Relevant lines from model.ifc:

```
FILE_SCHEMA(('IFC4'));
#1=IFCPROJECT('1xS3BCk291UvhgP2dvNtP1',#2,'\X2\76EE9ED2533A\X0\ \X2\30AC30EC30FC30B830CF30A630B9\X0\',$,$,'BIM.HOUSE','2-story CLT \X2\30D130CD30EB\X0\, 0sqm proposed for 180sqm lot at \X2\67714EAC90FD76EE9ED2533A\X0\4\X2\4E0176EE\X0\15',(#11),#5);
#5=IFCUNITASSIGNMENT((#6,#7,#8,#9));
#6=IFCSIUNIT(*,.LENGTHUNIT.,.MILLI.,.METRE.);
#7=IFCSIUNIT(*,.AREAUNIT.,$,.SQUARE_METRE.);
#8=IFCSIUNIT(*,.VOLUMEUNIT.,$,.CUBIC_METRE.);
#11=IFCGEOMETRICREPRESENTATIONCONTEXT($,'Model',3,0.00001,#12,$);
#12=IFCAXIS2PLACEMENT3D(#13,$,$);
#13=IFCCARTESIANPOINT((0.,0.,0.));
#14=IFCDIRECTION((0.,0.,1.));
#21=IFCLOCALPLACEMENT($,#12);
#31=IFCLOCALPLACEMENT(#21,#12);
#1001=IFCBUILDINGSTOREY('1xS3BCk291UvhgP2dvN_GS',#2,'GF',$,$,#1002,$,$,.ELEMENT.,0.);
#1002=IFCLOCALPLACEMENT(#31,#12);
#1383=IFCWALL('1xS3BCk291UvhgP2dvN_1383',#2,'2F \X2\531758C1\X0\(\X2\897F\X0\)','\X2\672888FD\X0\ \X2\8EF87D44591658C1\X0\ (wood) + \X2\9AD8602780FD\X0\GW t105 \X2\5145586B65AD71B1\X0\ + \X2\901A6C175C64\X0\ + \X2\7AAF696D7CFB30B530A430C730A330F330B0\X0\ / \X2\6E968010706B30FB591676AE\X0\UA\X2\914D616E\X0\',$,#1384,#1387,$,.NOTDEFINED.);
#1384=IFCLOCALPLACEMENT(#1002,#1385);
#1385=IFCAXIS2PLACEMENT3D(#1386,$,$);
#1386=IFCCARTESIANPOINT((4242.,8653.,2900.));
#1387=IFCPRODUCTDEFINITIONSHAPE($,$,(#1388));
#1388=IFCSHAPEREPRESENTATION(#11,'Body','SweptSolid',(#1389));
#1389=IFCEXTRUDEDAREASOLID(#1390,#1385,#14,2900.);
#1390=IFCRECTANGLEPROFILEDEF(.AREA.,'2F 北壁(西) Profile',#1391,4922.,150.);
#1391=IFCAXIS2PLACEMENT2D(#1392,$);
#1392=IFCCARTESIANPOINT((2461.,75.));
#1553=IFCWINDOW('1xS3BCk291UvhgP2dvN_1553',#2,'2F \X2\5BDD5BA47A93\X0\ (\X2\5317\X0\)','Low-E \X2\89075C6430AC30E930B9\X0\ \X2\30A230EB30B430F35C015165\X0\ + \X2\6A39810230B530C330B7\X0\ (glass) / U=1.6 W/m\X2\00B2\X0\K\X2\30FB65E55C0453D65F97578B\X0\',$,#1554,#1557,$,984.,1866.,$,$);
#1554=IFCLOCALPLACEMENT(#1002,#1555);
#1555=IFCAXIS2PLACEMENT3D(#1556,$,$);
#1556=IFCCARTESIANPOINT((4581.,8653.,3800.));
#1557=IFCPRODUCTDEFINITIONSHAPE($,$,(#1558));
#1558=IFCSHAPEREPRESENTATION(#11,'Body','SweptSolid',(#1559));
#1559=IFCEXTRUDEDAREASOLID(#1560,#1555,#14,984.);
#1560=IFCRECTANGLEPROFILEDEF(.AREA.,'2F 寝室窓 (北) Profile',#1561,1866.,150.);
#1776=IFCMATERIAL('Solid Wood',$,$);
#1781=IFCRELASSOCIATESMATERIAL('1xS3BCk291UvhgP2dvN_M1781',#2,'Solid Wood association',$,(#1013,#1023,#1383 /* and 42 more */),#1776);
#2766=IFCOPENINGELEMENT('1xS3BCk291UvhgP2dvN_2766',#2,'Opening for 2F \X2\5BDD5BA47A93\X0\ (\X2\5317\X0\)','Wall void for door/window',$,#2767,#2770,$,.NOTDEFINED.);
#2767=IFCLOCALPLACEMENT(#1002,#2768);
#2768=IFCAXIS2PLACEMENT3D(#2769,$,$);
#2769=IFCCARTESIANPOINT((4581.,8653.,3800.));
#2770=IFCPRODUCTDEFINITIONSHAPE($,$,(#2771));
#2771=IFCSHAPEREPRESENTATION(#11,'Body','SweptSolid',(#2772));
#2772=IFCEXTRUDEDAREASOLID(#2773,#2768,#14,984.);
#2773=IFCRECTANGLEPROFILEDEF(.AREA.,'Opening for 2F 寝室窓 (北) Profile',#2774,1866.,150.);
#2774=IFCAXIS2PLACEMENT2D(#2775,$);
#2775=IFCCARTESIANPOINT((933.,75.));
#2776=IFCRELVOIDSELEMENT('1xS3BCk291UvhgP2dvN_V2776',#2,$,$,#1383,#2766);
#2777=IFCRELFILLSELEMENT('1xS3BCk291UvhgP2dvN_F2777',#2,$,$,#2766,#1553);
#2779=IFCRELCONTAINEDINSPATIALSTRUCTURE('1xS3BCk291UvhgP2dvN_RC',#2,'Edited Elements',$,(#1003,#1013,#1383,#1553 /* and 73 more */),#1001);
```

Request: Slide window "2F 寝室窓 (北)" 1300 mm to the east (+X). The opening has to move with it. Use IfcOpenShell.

```python
import ifcopenshell
import ifcopenshell.api.geometry
import ifcopenshell.util.placement
import ifcopenshell.util.unit

model = ifcopenshell.open("model.ifc")
unit_scale = ifcopenshell.util.unit.calculate_unit_scale(model)

window = model.by_id(1553)
opening = window.FillsVoids[0].RelatingOpeningElement
wall = opening.VoidsElements[0].RelatingBuildingElement

wall_matrix = ifcopenshell.util.placement.get_local_placement(wall.ObjectPlacement)
shift = wall_matrix[:3, 0] * 1.3 / unit_scale
before = ifcopenshell.util.placement.get_local_placement(window.ObjectPlacement)[:3, 3].copy()

# The window is not placed relative to its opening, so move both.
for product in (opening, window):
    matrix = ifcopenshell.util.placement.get_local_placement(product.ObjectPlacement)
    matrix[:3, 3] += shift
    ifcopenshell.api.geometry.edit_object_placement(model, product=product, matrix=matrix, is_si=False)

after = ifcopenshell.util.placement.get_local_placement(window.ObjectPlacement)[:3, 3]
print("window moved by", (after - before).round(3) + 0.0)

model.write("model-out.ifc")
```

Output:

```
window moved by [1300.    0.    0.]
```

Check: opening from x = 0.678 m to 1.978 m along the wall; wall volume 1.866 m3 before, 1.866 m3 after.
